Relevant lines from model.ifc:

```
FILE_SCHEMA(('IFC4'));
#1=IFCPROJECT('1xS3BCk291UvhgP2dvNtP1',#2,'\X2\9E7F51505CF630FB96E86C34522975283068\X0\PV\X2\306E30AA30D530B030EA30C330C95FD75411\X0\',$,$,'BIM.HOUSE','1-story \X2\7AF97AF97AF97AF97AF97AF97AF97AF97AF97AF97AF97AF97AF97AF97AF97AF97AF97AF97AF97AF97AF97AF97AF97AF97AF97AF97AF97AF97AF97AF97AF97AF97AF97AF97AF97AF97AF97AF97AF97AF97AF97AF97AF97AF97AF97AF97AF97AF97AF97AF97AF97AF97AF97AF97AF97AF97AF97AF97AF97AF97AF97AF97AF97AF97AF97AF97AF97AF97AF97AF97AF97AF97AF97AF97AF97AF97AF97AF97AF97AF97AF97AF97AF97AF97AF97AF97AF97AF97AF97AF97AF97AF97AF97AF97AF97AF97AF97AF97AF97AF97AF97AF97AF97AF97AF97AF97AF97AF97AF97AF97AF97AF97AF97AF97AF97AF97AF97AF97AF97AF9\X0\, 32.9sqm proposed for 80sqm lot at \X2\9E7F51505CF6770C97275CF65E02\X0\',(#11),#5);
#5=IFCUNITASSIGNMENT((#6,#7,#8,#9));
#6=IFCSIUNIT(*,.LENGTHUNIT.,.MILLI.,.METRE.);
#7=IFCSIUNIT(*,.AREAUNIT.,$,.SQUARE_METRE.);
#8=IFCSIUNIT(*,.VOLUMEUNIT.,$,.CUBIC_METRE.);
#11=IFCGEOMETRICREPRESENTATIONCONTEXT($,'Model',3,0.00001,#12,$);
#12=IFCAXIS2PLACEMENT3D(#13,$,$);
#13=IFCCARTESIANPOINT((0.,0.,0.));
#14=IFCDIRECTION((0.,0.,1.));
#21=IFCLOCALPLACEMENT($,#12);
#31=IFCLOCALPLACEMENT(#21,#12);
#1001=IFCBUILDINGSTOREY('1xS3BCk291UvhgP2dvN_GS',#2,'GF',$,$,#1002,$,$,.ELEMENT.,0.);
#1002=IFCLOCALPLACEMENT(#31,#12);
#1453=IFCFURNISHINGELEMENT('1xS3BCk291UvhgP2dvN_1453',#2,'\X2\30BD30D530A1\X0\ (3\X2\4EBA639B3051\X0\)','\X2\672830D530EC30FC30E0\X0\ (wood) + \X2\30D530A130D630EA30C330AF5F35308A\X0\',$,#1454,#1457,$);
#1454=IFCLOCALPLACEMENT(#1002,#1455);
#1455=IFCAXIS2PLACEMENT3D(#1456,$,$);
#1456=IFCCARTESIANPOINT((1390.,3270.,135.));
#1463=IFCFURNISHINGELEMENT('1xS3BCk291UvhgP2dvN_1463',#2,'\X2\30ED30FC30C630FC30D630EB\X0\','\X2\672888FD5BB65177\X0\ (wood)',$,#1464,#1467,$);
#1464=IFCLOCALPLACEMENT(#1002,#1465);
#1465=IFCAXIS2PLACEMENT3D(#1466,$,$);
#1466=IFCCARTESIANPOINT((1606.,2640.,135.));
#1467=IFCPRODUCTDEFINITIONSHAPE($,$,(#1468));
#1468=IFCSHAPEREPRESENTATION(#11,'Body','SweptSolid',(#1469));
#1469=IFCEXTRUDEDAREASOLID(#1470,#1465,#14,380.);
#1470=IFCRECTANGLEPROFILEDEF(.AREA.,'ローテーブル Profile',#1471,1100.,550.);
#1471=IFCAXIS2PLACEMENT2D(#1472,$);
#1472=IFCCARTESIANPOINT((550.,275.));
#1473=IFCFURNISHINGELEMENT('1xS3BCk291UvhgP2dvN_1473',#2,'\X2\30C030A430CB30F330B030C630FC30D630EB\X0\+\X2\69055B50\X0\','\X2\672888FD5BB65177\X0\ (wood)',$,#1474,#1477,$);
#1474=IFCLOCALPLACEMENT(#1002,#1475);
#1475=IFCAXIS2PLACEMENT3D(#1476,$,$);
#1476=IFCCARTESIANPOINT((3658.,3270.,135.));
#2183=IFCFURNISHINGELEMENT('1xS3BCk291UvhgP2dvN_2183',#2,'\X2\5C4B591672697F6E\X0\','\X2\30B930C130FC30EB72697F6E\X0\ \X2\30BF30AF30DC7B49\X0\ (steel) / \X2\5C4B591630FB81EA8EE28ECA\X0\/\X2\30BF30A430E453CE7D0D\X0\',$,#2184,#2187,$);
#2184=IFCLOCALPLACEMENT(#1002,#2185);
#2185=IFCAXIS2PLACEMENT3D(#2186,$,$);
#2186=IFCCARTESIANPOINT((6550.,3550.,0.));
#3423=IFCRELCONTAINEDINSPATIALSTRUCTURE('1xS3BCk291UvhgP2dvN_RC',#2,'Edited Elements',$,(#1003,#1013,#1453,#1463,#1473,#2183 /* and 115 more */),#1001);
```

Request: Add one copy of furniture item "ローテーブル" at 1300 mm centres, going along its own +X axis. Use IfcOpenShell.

```python
import ifcopenshell
import ifcopenshell.api.geometry
import ifcopenshell.api.root
import ifcopenshell.util.element
import ifcopenshell.util.placement

model = ifcopenshell.open("model.ifc")


def reuse_history(source, copy):
    """copy_class also copies each property set's owner history, people and application; keep the originals."""
    for rel in copy.IsDefinedBy:
        if rel.is_a("IfcRelDefinesByProperties") and (history := rel.RelatingPropertyDefinition.OwnerHistory):
            rel.RelatingPropertyDefinition.OwnerHistory = source.OwnerHistory
            ifcopenshell.util.element.remove_deep2(model, history)


source = model.by_id(1463)
base = ifcopenshell.util.placement.get_local_placement(source.ObjectPlacement)
step = base[:3, 0] * 1300.0

for i in range(1, 2):
    copy = ifcopenshell.api.root.copy_class(model, product=source)
    copy.Representation = ifcopenshell.util.element.copy_deep(
        model, source.Representation, exclude=["IfcGeometricRepresentationContext", "IfcRepresentationMap"]
    )
    reuse_history(source, copy)
    matrix = base.copy()
    matrix[:3, 3] += i * step
    print("added at", matrix[:3, 3].round(3) + 0.0)
    ifcopenshell.api.geometry.edit_object_placement(model, product=copy, matrix=matrix, is_si=False)

model.write("model_edited.ifc")
```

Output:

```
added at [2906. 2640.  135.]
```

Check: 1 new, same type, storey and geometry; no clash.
